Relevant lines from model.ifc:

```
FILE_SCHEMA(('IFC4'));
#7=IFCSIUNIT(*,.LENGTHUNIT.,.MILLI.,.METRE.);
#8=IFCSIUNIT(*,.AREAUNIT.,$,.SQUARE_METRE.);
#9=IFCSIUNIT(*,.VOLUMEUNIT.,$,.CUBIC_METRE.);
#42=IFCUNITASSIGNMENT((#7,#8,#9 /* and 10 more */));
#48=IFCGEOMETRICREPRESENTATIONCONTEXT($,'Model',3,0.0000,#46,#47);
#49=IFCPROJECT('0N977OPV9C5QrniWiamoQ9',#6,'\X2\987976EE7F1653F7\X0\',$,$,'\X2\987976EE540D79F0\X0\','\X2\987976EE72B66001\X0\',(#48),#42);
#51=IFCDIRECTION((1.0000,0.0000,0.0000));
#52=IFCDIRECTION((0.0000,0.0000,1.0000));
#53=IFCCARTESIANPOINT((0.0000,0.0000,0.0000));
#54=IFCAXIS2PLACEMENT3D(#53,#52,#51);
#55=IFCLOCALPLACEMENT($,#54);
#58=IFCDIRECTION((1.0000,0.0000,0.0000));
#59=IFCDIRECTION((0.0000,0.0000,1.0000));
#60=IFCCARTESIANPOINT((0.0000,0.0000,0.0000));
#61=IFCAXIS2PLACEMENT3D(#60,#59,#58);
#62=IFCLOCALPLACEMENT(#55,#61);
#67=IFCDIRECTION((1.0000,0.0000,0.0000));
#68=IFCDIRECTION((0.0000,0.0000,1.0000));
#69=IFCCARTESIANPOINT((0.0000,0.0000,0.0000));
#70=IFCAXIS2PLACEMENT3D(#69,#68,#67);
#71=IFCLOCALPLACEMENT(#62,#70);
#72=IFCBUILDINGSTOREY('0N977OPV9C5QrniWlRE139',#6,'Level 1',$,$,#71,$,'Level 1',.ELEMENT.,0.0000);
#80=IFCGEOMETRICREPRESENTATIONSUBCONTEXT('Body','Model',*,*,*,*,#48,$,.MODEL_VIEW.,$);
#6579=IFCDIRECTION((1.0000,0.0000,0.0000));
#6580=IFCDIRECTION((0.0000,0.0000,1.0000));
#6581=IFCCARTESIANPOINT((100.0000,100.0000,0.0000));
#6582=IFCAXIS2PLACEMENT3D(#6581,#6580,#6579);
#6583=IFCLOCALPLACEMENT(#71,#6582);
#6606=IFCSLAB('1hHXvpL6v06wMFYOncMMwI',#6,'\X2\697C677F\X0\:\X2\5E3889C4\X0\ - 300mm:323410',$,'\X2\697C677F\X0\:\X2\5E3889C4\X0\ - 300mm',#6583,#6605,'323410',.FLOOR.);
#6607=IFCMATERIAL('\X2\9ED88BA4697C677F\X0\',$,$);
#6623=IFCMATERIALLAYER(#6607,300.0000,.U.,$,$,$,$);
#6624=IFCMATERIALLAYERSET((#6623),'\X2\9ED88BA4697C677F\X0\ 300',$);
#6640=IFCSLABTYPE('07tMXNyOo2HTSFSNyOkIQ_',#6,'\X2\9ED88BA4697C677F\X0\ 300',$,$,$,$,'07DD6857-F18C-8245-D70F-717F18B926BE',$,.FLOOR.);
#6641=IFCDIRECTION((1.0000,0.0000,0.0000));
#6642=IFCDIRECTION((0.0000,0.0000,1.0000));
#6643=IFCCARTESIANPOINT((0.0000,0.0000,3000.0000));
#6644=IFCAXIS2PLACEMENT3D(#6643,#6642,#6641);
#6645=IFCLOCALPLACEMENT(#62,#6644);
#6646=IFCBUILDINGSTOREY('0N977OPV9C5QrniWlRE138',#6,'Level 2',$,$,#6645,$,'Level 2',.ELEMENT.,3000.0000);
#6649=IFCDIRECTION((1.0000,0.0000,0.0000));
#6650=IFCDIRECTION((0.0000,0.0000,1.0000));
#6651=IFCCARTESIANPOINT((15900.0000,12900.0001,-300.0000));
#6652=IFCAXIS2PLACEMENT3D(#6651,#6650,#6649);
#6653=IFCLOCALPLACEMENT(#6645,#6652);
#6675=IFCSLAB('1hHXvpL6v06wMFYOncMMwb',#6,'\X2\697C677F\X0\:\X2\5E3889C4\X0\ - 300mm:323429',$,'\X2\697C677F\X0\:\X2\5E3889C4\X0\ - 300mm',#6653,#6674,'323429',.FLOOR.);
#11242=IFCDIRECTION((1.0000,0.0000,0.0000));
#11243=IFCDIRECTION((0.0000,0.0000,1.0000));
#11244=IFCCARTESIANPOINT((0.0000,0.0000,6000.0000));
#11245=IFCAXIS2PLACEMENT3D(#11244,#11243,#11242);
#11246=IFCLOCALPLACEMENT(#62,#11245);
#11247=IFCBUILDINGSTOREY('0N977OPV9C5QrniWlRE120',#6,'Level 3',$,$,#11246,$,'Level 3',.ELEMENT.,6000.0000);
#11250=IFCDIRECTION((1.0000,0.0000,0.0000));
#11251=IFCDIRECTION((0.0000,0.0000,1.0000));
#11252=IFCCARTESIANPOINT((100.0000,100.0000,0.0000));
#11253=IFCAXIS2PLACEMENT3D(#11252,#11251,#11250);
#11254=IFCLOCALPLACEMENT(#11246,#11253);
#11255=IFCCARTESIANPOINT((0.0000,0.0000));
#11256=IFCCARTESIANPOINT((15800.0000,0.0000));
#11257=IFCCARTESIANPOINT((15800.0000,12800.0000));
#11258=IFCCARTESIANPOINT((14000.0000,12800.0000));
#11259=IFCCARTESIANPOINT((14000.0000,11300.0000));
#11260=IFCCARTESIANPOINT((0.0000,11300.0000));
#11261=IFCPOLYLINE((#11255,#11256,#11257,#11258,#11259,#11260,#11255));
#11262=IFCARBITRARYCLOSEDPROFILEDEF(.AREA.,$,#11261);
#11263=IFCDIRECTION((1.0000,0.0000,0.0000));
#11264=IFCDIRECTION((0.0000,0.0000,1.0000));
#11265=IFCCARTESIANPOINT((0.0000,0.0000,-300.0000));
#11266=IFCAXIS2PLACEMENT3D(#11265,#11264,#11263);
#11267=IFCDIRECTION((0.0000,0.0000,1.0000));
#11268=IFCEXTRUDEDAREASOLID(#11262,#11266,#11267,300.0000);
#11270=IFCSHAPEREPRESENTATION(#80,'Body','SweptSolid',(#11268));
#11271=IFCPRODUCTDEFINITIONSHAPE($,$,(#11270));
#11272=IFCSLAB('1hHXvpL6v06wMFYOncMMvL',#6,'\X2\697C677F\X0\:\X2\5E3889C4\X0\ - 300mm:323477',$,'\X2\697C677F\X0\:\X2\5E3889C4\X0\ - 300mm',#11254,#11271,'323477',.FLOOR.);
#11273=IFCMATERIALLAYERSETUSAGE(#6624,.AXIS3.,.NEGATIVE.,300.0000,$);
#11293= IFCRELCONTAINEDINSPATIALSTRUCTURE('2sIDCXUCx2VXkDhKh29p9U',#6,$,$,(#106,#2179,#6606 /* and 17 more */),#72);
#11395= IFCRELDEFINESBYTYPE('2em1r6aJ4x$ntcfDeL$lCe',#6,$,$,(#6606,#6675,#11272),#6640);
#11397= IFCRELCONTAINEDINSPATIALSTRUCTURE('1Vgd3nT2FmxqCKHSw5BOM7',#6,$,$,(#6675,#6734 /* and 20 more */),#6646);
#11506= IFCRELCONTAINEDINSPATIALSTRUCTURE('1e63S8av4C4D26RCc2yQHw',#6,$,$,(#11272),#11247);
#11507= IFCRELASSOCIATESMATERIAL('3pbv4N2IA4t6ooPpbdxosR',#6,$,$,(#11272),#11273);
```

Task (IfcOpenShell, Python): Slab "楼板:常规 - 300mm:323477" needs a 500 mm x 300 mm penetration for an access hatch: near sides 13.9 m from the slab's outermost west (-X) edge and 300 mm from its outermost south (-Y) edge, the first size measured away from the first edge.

```python
import numpy as np
import ifcopenshell
import ifcopenshell.api.feature
import ifcopenshell.api.geometry
import ifcopenshell.api.root
import ifcopenshell.geom
import ifcopenshell.util.placement
import ifcopenshell.util.representation
import ifcopenshell.util.shape
import ifcopenshell.util.unit

model = ifcopenshell.open("model.ifc")
unit_scale = ifcopenshell.util.unit.calculate_unit_scale(model)
settings = ifcopenshell.geom.settings()


def volume(element):
    """Net volume in cubic metres, openings subtracted."""
    shape = ifcopenshell.geom.create_shape(settings, element)
    return ifcopenshell.util.shape.get_volume(shape.geometry)


slab = model.by_guid("1hHXvpL6v06wMFYOncMMvL")
before = volume(slab)

# Extent in the slab's own axes, in metres. The edges named are its -X and -Y sides.
slab_shape = ifcopenshell.geom.create_shape(settings, slab)
vertices = ifcopenshell.util.shape.get_vertices(slab_shape.geometry)
x_min, y_min, bottom = vertices.min(axis=0)
top = vertices[:, 2].max()

opening = ifcopenshell.api.root.create_entity(model, ifc_class="IfcOpeningElement", name="Access hatch opening", predefined_type="OPENING")
context = ifcopenshell.util.representation.get_context(model, "Model", "Body", "MODEL_VIEW")
width, depth = 0.5, 0.3
outline = [(0.0, 0.0), (width, 0.0), (width, depth), (0.0, depth), (0.0, 0.0)]
# Overshoot both faces by 50 mm so the cut is clean.
shape = ifcopenshell.api.geometry.add_slab_representation(
    model, context=context, depth=top - bottom + 0.1, polyline=outline
)
ifcopenshell.api.geometry.assign_representation(model, product=opening, representation=shape)

matrix = ifcopenshell.util.placement.get_local_placement(slab.ObjectPlacement)
matrix[:, 3] = matrix @ np.append(np.array([x_min + 13.9, y_min + 0.3, bottom - 0.05]) / unit_scale, 1.0)
ifcopenshell.api.geometry.edit_object_placement(model, product=opening, matrix=matrix, is_si=False)
ifcopenshell.api.feature.add_feature(model, feature=opening, element=slab)

after = volume(slab)

print(f"slab volume {before:.3f} -> {after:.3f} m3")

model.write("model_v2.ifc")
```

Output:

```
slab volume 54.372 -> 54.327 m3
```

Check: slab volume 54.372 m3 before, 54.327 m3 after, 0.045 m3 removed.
